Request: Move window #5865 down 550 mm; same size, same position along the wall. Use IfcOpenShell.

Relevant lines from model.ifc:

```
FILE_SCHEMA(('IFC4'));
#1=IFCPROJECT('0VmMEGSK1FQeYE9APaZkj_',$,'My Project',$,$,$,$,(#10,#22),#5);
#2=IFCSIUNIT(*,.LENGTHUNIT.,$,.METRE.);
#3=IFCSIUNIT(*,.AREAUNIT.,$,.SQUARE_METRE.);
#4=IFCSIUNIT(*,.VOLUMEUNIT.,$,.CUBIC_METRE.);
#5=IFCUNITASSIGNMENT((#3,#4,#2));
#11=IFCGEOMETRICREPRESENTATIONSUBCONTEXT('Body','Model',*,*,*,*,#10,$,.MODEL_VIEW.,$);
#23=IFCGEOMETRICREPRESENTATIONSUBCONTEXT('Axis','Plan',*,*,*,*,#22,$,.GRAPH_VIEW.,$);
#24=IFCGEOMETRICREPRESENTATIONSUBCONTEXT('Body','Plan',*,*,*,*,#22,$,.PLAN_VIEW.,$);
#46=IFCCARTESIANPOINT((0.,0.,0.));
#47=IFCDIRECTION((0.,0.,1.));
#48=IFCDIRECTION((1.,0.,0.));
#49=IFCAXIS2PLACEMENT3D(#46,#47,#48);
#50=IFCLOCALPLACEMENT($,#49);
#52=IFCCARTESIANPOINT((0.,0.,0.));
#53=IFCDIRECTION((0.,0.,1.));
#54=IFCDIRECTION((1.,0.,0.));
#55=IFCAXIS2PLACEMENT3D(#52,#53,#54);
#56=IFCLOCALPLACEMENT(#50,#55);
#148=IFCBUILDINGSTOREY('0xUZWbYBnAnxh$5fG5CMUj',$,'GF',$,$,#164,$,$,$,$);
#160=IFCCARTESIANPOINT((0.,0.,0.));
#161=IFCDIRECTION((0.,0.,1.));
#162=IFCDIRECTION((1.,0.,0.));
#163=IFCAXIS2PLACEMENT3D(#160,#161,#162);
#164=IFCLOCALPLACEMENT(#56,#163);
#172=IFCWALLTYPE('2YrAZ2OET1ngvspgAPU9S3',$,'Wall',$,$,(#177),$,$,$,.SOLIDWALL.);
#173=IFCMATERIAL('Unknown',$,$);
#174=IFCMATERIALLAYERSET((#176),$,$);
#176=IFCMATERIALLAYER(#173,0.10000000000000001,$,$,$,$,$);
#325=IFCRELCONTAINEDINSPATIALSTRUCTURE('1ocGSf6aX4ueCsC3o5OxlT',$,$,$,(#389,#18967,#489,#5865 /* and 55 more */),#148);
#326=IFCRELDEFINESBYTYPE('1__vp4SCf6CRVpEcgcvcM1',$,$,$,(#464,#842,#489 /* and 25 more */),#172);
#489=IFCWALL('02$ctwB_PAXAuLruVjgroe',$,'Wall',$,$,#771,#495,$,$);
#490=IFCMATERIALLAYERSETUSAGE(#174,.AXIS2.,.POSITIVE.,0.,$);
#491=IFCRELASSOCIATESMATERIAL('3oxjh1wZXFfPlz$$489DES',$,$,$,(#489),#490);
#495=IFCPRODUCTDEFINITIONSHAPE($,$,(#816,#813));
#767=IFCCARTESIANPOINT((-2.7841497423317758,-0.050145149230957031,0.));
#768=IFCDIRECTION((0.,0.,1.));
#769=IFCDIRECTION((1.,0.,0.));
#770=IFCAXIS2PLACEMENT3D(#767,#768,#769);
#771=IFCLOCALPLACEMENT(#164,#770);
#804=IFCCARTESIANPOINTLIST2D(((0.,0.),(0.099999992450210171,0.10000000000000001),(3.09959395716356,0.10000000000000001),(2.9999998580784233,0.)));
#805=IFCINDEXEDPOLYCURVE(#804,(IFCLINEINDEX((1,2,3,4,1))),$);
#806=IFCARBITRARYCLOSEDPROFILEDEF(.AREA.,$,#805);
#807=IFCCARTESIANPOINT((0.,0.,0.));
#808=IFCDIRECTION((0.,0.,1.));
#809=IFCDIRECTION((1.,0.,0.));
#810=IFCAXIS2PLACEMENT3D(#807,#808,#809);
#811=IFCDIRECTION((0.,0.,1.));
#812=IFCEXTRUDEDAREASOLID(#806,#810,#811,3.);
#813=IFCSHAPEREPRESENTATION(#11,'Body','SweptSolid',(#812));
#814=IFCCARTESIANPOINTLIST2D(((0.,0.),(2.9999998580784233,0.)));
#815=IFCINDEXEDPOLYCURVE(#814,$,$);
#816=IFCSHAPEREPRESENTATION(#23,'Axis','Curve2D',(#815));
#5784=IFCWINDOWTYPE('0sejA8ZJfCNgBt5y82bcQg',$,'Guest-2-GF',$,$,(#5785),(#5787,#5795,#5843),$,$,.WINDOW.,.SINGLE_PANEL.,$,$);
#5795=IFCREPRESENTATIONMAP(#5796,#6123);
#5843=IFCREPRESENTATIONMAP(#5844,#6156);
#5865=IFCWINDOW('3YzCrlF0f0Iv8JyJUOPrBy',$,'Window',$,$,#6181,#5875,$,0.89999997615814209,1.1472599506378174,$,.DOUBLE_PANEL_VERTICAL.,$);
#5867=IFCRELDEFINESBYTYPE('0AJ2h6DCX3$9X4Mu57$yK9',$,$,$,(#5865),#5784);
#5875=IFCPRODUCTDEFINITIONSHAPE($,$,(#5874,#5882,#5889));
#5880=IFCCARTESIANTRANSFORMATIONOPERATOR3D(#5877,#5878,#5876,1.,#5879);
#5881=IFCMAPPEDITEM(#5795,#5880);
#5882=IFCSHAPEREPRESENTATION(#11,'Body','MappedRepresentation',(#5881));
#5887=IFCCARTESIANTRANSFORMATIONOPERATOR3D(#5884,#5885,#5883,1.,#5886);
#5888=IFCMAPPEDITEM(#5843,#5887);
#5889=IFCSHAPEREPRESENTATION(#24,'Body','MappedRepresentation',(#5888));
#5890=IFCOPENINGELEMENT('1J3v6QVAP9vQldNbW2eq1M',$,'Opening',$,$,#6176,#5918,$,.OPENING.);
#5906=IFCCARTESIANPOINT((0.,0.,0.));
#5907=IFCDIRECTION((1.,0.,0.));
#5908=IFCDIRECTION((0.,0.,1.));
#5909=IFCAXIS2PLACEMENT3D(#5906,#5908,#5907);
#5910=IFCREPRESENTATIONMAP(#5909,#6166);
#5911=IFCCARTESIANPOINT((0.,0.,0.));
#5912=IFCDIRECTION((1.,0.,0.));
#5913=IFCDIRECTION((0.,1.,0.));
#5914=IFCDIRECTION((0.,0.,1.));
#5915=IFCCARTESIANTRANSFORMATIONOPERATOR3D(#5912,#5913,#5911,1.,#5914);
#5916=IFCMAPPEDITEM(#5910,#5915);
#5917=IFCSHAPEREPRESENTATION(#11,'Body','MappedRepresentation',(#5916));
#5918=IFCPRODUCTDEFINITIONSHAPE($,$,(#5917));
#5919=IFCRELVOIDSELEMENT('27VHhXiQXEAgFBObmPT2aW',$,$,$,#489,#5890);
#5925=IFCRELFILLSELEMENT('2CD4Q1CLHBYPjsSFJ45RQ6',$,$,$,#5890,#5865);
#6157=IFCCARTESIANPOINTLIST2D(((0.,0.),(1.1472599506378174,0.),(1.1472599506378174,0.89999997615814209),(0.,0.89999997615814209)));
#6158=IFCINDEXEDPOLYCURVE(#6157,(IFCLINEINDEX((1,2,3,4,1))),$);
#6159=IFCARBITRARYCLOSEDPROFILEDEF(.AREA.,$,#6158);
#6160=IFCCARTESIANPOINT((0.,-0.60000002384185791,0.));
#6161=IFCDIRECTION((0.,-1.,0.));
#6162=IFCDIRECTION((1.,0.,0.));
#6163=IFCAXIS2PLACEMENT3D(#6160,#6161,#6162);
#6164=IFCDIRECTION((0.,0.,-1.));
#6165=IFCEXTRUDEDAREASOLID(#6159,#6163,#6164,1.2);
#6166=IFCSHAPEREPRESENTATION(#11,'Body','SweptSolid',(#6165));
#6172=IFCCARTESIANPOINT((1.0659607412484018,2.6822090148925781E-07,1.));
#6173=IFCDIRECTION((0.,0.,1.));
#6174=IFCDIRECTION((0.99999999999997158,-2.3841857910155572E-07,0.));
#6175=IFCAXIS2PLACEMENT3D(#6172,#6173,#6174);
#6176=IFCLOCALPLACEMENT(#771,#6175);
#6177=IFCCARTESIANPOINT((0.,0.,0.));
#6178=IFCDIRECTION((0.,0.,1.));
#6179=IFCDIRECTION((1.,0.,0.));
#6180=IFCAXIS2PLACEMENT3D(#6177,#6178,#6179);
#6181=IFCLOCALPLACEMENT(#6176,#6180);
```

```python
import numpy as np
import ifcopenshell
import ifcopenshell.api.geometry
import ifcopenshell.util.placement
import ifcopenshell.util.unit

model = ifcopenshell.open("model.ifc")
unit_scale = ifcopenshell.util.unit.calculate_unit_scale(model)

window = model.by_guid("3YzCrlF0f0Iv8JyJUOPrBy")
opening = window.FillsVoids[0].RelatingOpeningElement
dz = -0.55

shift = np.array([0.0, 0.0, dz])
# The window is placed relative to its opening, so it follows when the opening moves.
matrix = ifcopenshell.util.placement.get_local_placement(opening.ObjectPlacement)
matrix[:3, 3] += shift
ifcopenshell.api.geometry.edit_object_placement(
    model, product=opening, matrix=matrix, is_si=False, should_transform_children=True
)

print(f"moved by {dz * unit_scale:+.3f} m")

model.write("model_v2.ifc")
```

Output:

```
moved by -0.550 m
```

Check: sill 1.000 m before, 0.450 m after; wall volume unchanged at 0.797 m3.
